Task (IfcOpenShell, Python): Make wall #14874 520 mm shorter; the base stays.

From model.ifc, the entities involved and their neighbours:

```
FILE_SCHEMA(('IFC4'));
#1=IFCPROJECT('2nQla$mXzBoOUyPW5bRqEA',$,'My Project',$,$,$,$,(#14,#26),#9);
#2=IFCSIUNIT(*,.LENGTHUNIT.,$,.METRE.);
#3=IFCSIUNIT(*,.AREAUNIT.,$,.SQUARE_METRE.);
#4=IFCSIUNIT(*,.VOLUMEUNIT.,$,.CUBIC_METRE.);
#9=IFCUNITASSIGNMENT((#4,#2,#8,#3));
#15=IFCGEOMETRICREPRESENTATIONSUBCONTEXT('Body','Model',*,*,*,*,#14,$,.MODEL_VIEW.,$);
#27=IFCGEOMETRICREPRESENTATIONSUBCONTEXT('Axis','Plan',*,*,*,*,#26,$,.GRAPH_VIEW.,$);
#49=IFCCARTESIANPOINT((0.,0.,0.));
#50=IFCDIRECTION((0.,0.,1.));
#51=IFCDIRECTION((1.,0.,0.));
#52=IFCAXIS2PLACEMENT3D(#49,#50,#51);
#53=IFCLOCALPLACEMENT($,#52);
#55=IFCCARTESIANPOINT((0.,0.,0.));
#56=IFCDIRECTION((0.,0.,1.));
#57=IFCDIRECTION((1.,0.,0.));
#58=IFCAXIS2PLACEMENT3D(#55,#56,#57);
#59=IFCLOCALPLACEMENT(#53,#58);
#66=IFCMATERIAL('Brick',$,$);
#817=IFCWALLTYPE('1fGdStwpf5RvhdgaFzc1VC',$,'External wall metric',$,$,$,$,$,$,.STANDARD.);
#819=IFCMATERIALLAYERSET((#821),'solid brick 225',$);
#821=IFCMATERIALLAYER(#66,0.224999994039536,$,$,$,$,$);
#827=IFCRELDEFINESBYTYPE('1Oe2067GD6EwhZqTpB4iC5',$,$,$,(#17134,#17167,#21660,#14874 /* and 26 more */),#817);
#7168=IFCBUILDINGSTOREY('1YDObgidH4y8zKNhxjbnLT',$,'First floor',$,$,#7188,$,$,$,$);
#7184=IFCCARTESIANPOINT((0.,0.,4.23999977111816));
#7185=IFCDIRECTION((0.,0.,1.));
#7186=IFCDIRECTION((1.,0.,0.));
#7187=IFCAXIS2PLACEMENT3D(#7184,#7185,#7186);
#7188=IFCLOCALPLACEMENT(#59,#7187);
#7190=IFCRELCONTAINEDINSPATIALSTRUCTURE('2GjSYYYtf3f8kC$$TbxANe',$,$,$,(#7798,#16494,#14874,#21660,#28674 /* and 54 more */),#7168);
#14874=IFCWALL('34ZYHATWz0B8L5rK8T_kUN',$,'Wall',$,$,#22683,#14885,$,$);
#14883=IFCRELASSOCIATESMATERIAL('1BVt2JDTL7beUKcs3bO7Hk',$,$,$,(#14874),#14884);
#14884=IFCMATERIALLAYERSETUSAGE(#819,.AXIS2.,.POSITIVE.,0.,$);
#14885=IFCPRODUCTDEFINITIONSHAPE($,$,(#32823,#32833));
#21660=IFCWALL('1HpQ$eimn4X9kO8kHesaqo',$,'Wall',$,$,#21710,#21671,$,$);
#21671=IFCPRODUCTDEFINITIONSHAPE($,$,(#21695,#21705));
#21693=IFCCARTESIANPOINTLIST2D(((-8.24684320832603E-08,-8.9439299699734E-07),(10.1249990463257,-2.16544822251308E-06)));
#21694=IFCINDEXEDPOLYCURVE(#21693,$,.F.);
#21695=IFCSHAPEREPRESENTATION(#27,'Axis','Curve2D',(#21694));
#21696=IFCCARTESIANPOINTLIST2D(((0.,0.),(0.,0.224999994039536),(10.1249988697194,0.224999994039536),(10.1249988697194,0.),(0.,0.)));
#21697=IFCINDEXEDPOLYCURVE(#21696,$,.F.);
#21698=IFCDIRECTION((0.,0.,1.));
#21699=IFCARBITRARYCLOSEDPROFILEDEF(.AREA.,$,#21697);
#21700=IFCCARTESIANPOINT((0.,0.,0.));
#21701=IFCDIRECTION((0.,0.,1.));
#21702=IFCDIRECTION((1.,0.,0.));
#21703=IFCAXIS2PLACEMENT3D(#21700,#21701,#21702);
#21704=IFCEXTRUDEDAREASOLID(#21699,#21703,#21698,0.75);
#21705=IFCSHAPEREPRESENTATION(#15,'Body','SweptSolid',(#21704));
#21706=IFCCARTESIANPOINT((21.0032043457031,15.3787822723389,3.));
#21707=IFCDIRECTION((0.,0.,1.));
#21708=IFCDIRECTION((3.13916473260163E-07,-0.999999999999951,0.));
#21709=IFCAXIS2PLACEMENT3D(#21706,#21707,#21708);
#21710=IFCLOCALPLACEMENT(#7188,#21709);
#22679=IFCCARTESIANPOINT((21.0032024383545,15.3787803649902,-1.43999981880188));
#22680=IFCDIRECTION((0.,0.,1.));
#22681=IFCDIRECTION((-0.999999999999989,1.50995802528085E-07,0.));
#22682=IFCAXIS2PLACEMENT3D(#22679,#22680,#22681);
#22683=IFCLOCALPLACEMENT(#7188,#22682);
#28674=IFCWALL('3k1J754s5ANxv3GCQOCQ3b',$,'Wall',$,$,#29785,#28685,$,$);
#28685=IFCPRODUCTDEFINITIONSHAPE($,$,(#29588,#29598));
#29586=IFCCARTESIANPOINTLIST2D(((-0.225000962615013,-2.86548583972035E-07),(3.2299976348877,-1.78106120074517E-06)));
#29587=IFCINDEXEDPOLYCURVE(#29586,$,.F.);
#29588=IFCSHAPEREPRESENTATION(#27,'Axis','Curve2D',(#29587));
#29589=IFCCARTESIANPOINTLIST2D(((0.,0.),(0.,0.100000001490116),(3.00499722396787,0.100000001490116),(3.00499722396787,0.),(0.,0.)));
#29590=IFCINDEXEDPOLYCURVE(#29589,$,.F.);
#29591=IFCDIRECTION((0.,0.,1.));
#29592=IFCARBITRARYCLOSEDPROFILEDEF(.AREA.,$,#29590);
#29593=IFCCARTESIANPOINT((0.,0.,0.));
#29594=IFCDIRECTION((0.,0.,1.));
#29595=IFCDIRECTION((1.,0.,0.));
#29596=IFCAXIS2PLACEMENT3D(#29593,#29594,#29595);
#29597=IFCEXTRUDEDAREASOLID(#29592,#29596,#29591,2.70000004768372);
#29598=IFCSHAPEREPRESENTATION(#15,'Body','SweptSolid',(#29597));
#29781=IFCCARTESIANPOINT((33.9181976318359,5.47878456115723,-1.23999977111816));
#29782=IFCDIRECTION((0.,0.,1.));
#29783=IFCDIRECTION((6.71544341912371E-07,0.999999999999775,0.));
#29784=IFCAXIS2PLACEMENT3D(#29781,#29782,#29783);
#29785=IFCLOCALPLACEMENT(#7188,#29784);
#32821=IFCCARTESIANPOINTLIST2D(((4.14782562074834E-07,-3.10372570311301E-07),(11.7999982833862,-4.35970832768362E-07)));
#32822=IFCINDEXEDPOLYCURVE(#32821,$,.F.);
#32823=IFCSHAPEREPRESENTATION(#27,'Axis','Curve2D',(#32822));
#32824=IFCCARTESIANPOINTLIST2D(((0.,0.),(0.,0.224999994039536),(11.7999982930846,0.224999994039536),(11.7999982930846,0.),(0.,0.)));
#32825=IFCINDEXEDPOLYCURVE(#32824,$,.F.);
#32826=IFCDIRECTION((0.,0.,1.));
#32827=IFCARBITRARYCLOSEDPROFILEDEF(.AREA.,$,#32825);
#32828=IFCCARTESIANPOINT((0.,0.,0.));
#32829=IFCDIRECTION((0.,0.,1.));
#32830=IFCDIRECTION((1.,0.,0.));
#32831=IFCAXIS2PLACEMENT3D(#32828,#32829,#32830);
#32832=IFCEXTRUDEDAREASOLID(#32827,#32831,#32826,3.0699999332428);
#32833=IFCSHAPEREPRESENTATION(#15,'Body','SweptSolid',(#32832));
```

```python
import ifcopenshell
import ifcopenshell.geom
import ifcopenshell.util.representation
import ifcopenshell.util.shape

model = ifcopenshell.open("model.ifc")
settings = ifcopenshell.geom.settings()


def volume(element):
    """Net volume in cubic metres, openings subtracted."""
    shape = ifcopenshell.geom.create_shape(settings, element)
    return ifcopenshell.util.shape.get_volume(shape.geometry)


wall = model.by_guid("34ZYHATWz0B8L5rK8T_kUN")
before = volume(wall)

body = ifcopenshell.util.representation.get_representation(wall, "Model", "Body")
solid = body.Items[0]
old_height = solid.Depth
solid.Depth -= 0.52
after = volume(wall)

print(f"height {old_height:g} -> {solid.Depth:g}, volume {before:.3f} -> {after:.3f} m3")

model.write("model-out.ifc")
```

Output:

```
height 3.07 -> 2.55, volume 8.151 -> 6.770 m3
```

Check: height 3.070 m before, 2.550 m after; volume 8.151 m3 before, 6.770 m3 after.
